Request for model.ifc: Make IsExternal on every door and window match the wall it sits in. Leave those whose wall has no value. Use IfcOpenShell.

First a look at what the model holds.

```python
import ifcopenshell
import ifcopenshell.util.element

model = ifcopenshell.open("model.ifc")
print(model.schema)
seen = {}
for e in model.by_type("IfcDoor") + model.by_type("IfcWindow"):
    if not e.FillsVoids:
        continue
    host = e.FillsVoids[0].RelatingOpeningElement.VoidsElements[0].RelatingBuildingElement
    own = ifcopenshell.util.element.get_pset(e, f"Pset_{e.is_a()[3:].removesuffix('StandardCase')}Common", "IsExternal")
    wall = ifcopenshell.util.element.get_pset(host, "Pset_WallCommon", "IsExternal")
    seen[e.is_a(), own, wall] = seen.get((e.is_a(), own, wall), 0) + 1
for (cls, own, wall), count in sorted(seen.items(), key=str):
    print(count, cls, "IsExternal:", own, "| host wall:", wall)
```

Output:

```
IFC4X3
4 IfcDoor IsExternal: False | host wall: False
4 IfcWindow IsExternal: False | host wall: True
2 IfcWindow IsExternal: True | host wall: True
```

```python
import ifcopenshell
import ifcopenshell.api.pset
import ifcopenshell.util.element

model = ifcopenshell.open("model.ifc")

count = 0
for ifc_class, pset_name in (("IfcDoor", "Pset_DoorCommon"), ("IfcWindow", "Pset_WindowCommon")):
    for e in model.by_type(ifc_class):
        if not e.FillsVoids:
            continue
        host = e.FillsVoids[0].RelatingOpeningElement.VoidsElements[0].RelatingBuildingElement
        external = ifcopenshell.util.element.get_pset(host, "Pset_WallCommon", "IsExternal")
        if external is None or ifcopenshell.util.element.get_pset(e, pset_name, "IsExternal") == external:
            continue
        pset = ifcopenshell.api.pset.add_pset(model, product=e, name=pset_name)
        ifcopenshell.api.pset.edit_pset(model, pset=pset, properties={"IsExternal": external})
        count += 1

print(count, "updated")

model.write("model_updated.ifc")
```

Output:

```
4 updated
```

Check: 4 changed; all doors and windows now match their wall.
